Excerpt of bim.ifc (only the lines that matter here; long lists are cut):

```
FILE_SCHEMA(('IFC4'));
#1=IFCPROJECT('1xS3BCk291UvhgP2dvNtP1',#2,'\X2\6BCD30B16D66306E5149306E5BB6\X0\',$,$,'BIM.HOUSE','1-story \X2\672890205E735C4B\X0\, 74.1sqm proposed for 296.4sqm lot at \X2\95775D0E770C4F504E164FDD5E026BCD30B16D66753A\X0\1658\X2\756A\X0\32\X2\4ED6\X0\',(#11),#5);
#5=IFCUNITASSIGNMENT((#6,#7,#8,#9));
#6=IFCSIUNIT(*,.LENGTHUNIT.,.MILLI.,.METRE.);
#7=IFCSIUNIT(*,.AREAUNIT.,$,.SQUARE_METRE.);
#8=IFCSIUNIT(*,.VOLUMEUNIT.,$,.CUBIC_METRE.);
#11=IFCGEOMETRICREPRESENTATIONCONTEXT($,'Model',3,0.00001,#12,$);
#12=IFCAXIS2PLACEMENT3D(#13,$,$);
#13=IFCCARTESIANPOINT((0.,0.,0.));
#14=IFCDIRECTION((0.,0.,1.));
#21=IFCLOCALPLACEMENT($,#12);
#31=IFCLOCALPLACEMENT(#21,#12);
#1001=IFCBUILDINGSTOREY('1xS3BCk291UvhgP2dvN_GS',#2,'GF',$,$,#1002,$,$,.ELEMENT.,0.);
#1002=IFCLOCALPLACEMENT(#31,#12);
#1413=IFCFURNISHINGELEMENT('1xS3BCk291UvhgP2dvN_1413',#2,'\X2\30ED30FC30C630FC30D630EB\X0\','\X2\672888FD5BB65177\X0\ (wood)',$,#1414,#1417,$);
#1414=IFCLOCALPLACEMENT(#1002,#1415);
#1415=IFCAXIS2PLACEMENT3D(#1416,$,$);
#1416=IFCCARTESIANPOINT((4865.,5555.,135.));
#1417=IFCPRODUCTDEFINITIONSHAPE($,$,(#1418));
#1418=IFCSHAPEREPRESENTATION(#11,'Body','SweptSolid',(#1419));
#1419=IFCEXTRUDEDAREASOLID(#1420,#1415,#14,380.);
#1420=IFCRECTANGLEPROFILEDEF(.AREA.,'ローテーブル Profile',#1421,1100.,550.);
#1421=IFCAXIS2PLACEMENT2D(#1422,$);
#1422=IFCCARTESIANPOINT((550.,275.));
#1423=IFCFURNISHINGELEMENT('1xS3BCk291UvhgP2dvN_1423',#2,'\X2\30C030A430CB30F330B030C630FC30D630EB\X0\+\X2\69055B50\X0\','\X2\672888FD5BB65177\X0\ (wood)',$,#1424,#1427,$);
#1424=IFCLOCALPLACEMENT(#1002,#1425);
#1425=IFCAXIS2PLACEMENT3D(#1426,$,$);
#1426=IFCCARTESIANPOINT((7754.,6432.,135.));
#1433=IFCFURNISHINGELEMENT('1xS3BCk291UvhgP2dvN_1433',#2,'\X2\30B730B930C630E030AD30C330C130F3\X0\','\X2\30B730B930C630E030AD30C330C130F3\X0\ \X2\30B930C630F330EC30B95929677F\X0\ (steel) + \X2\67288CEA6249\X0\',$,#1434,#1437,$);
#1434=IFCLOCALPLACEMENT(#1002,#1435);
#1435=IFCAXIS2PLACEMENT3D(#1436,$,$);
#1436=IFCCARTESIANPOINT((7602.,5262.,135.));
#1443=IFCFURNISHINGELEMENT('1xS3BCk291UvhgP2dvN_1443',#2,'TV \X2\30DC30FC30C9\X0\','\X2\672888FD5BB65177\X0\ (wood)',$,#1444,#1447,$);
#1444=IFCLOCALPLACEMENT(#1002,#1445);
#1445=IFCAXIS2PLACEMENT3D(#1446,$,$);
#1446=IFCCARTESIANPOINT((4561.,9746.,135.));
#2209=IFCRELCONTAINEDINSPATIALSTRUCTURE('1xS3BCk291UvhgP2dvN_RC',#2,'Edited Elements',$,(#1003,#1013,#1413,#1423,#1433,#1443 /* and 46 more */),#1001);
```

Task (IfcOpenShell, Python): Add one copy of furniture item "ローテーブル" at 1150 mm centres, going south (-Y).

```python
import numpy as np
import ifcopenshell
import ifcopenshell.api.geometry
import ifcopenshell.api.root
import ifcopenshell.util.element
import ifcopenshell.util.placement

model = ifcopenshell.open("bim.ifc")


def reuse_history(source, copy):
    """copy_class also copies each property set's owner history, people and application; keep the originals."""
    for rel in copy.IsDefinedBy:
        if rel.is_a("IfcRelDefinesByProperties") and (history := rel.RelatingPropertyDefinition.OwnerHistory):
            rel.RelatingPropertyDefinition.OwnerHistory = source.OwnerHistory
            ifcopenshell.util.element.remove_deep2(model, history)


source = model.by_guid("1xS3BCk291UvhgP2dvN_1413")
base = ifcopenshell.util.placement.get_local_placement(source.ObjectPlacement)
step = np.array([0.0, -1.0, 0.0]) * 1150.0

for i in range(1, 2):
    copy = ifcopenshell.api.root.copy_class(model, product=source)
    copy.Representation = ifcopenshell.util.element.copy_deep(
        model, source.Representation, exclude=["IfcGeometricRepresentationContext", "IfcRepresentationMap"]
    )
    reuse_history(source, copy)
    matrix = base.copy()
    matrix[:3, 3] += i * step
    print("added at", matrix[:3, 3].round(3) + 0.0)
    ifcopenshell.api.geometry.edit_object_placement(model, product=copy, matrix=matrix, is_si=False)

model.write("bim_updated.ifc")
```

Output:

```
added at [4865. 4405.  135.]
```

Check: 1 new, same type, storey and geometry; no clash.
